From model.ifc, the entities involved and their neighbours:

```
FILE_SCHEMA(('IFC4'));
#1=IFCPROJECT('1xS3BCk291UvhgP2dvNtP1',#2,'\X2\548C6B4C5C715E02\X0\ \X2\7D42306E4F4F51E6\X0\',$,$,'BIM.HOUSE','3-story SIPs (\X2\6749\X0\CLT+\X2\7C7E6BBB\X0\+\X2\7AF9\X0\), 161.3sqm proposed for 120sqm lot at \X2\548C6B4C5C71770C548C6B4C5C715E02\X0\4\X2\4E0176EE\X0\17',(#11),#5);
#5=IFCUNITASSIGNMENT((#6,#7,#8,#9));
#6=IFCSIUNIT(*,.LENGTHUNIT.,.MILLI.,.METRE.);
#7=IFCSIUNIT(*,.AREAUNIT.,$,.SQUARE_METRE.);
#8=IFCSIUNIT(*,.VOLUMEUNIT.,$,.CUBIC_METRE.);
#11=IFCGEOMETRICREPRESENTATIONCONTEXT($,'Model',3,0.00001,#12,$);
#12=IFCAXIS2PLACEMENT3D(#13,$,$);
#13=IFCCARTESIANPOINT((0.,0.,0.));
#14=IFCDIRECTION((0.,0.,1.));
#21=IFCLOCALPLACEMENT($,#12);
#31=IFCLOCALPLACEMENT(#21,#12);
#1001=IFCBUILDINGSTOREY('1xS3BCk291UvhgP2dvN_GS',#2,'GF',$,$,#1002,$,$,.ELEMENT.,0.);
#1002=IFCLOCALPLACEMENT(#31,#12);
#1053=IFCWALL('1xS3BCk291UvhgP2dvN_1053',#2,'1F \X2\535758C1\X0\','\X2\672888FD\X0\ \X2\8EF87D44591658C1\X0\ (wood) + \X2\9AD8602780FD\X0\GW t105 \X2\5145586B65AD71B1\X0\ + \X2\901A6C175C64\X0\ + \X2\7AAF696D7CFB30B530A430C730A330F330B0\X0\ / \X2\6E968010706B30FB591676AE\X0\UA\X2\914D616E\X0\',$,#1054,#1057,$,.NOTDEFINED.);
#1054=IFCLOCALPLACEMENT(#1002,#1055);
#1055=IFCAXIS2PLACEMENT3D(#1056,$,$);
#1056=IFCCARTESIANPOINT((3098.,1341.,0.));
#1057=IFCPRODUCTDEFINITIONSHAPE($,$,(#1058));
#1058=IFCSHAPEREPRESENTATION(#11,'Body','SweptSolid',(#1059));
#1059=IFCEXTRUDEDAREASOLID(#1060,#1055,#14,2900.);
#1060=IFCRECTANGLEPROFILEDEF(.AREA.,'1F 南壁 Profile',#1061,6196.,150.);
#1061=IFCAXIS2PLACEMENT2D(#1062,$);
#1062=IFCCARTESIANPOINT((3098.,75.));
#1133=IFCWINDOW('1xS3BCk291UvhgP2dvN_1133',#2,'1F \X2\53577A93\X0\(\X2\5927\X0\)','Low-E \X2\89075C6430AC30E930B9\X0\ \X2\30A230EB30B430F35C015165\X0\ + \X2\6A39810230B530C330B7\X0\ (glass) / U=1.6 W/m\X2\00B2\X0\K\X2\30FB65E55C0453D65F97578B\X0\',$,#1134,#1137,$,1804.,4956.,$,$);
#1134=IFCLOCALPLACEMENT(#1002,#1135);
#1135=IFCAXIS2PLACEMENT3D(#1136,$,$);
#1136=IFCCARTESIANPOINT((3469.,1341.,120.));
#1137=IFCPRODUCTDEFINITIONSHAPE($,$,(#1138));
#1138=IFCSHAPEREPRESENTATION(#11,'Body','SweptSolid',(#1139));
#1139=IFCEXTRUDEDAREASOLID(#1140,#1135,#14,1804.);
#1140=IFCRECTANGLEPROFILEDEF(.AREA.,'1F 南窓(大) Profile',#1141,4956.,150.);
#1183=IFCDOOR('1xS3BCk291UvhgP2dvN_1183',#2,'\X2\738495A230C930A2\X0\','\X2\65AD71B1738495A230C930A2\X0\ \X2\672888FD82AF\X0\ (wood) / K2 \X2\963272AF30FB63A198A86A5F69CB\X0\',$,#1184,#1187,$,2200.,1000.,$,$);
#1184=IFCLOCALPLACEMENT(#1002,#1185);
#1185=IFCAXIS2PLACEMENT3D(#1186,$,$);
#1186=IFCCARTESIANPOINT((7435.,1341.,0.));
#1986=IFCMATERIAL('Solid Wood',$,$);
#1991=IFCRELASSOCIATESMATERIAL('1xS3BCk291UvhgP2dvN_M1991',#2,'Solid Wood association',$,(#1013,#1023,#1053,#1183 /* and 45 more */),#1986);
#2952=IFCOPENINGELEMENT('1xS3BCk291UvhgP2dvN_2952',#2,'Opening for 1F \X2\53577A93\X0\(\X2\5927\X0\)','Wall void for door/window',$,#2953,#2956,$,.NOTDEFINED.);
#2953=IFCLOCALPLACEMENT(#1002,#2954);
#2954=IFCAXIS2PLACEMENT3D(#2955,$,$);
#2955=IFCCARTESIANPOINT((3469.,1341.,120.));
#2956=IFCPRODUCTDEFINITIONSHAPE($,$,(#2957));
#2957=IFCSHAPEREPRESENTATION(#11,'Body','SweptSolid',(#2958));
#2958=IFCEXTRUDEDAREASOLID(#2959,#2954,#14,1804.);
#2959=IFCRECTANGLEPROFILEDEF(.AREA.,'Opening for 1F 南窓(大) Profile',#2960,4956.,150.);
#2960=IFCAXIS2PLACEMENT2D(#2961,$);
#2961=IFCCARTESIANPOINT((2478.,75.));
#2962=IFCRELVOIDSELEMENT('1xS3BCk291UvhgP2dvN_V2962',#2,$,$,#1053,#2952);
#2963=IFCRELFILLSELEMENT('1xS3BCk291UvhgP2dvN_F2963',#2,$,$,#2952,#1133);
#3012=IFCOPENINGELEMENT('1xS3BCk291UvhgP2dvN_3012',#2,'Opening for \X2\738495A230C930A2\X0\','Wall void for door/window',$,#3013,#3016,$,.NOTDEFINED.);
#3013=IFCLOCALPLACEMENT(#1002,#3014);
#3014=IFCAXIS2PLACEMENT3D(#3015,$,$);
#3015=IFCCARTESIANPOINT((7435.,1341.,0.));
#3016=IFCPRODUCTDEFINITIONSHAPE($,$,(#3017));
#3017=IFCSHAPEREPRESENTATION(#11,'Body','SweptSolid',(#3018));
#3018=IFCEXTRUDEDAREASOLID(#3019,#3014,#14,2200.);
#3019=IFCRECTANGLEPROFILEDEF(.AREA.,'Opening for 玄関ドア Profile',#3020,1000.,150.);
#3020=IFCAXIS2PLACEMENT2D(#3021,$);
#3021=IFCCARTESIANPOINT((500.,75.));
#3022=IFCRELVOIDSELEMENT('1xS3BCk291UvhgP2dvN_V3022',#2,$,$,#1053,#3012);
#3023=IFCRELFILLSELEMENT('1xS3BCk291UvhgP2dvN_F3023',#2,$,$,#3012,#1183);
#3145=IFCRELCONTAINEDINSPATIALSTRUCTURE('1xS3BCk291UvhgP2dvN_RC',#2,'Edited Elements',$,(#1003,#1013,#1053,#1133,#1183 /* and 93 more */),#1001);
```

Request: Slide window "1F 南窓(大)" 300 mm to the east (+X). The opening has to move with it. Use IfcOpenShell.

```python
import ifcopenshell
import ifcopenshell.api.geometry
import ifcopenshell.util.placement
import ifcopenshell.util.unit

model = ifcopenshell.open("model.ifc")
unit_scale = ifcopenshell.util.unit.calculate_unit_scale(model)

window = model.by_guid("1xS3BCk291UvhgP2dvN_1133")
opening = window.FillsVoids[0].RelatingOpeningElement
wall = opening.VoidsElements[0].RelatingBuildingElement

wall_matrix = ifcopenshell.util.placement.get_local_placement(wall.ObjectPlacement)
shift = wall_matrix[:3, 0] * 0.3 / unit_scale
before = ifcopenshell.util.placement.get_local_placement(window.ObjectPlacement)[:3, 3].copy()

# The window is not placed relative to its opening, so move both.
for product in (opening, window):
    matrix = ifcopenshell.util.placement.get_local_placement(product.ObjectPlacement)
    matrix[:3, 3] += shift
    ifcopenshell.api.geometry.edit_object_placement(model, product=product, matrix=matrix, is_si=False)

after = ifcopenshell.util.placement.get_local_placement(window.ObjectPlacement)[:3, 3]
print("window moved by", (after - before).round(3) + 0.0)

model.write("model_edited.ifc")
```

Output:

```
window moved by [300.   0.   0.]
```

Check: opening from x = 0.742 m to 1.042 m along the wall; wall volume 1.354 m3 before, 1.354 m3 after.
